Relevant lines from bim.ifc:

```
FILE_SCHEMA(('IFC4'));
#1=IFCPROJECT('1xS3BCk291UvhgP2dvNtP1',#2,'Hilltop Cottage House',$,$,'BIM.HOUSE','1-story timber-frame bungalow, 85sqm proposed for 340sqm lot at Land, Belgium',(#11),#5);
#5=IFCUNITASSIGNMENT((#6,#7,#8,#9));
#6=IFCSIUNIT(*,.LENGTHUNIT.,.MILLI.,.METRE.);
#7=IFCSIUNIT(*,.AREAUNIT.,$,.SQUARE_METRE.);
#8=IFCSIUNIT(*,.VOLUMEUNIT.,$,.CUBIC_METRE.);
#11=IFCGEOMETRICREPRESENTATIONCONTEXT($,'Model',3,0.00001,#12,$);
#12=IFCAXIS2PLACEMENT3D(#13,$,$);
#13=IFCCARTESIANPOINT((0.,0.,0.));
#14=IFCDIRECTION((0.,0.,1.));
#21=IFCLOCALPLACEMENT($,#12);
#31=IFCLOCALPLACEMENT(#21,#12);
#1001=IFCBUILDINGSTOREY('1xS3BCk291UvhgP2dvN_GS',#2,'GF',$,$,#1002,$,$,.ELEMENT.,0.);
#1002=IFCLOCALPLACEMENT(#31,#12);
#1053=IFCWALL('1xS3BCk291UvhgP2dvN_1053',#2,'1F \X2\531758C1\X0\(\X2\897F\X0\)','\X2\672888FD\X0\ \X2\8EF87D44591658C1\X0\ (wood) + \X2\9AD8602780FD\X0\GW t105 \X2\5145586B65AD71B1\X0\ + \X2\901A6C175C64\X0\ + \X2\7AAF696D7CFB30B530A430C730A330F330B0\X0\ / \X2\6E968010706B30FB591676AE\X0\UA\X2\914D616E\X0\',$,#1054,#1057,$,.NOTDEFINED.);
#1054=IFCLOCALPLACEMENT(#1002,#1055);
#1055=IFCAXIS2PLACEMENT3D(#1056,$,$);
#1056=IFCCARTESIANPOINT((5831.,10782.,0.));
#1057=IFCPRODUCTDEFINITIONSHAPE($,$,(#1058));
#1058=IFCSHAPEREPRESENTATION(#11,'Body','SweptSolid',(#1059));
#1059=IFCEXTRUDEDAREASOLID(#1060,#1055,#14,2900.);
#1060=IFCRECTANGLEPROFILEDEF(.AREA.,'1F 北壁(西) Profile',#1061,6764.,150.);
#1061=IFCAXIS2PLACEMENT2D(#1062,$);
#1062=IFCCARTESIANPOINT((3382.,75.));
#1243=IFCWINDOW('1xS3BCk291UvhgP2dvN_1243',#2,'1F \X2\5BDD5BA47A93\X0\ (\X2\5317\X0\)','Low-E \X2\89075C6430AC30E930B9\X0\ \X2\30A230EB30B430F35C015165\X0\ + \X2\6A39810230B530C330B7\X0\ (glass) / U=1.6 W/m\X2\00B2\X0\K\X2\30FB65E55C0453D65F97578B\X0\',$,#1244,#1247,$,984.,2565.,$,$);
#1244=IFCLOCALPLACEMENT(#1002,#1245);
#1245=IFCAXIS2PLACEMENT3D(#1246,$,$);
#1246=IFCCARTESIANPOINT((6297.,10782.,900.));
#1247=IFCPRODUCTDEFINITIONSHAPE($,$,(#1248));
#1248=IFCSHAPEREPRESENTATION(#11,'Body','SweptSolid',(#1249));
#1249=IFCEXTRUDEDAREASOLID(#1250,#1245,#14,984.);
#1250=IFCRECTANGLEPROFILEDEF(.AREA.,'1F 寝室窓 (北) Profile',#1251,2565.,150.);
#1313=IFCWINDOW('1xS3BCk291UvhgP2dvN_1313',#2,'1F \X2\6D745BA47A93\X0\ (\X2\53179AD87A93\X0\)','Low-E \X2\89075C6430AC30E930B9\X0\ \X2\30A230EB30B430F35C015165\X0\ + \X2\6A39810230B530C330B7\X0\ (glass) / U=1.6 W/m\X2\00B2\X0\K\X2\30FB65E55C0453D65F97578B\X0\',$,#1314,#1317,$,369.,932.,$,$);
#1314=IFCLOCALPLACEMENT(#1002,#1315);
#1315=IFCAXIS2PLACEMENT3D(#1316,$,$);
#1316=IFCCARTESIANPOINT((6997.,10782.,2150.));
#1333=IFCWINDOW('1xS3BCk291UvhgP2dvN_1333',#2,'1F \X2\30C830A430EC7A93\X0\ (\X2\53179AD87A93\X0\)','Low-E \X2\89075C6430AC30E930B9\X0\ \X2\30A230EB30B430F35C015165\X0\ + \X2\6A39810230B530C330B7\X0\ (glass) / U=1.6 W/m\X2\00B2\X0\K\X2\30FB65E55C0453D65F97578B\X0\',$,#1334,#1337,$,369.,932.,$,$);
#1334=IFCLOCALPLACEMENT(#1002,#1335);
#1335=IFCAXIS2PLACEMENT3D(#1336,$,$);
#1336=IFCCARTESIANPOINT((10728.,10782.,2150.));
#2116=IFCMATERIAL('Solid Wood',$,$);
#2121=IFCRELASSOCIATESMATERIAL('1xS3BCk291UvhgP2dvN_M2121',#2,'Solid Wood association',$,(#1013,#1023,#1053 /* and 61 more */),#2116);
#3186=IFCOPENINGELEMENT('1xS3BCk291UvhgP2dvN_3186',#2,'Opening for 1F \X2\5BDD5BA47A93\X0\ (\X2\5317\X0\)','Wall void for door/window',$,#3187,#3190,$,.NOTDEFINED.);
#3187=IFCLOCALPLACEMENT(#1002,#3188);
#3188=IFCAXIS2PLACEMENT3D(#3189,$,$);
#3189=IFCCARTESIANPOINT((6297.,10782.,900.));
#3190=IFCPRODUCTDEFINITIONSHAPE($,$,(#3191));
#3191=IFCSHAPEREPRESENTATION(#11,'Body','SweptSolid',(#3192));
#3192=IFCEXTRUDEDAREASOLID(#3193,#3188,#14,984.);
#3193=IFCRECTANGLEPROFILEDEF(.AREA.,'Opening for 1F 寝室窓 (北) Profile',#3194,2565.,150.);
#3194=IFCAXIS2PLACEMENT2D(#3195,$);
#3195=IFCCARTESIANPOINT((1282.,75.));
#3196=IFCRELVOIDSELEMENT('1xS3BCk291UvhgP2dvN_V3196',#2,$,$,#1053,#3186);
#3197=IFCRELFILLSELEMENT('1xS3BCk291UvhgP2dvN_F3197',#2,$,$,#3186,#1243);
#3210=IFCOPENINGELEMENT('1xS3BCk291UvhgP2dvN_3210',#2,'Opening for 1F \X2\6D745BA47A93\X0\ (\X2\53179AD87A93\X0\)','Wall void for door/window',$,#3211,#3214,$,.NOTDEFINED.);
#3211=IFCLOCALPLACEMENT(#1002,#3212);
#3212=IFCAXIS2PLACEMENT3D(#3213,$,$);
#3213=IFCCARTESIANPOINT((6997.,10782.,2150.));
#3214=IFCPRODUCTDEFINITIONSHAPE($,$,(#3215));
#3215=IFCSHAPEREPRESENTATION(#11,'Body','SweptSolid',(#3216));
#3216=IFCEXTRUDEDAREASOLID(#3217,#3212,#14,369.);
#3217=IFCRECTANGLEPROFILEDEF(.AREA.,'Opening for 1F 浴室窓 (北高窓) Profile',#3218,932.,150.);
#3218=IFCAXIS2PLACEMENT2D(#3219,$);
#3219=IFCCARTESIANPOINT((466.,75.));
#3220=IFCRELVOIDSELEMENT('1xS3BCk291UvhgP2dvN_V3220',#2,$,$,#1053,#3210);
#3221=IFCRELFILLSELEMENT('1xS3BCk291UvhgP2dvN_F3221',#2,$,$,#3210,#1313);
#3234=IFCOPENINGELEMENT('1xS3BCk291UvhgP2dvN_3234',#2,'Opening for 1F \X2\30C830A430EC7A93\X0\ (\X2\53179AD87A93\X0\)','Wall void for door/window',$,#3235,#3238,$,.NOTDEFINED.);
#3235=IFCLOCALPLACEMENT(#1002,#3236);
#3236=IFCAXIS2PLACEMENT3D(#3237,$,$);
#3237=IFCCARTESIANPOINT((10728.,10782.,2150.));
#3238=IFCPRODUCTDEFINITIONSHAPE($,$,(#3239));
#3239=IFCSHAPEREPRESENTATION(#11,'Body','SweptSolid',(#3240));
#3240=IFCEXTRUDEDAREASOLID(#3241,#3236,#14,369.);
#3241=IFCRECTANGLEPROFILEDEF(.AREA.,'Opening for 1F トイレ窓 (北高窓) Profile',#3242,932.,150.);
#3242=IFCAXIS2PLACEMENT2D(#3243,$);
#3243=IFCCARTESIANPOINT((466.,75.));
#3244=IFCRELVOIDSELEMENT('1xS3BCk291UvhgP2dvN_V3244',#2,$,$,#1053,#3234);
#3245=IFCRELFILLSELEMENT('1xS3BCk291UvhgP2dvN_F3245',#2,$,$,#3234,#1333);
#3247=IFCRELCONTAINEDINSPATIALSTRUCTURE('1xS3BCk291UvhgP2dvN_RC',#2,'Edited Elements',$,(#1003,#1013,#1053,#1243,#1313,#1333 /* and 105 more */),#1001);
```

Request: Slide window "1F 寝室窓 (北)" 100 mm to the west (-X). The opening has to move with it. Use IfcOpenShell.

```python
import ifcopenshell
import ifcopenshell.api.geometry
import ifcopenshell.util.placement

model = ifcopenshell.open("bim.ifc")

window = model.by_guid("1xS3BCk291UvhgP2dvN_1243")
opening = window.FillsVoids[0].RelatingOpeningElement
wall = opening.VoidsElements[0].RelatingBuildingElement

wall_matrix = ifcopenshell.util.placement.get_local_placement(wall.ObjectPlacement)
shift = wall_matrix[:3, 0] * -100.0
before = ifcopenshell.util.placement.get_local_placement(window.ObjectPlacement)[:3, 3].copy()

# The window is not placed relative to its opening, so move both.
for product in (opening, window):
    matrix = ifcopenshell.util.placement.get_local_placement(product.ObjectPlacement)
    matrix[:3, 3] += shift
    ifcopenshell.api.geometry.edit_object_placement(model, product=product, matrix=matrix, is_si=False)

after = ifcopenshell.util.placement.get_local_placement(window.ObjectPlacement)[:3, 3]
print("window moved by", (after - before).round(3) + 0.0)

model.write("bim_rev.ifc")
```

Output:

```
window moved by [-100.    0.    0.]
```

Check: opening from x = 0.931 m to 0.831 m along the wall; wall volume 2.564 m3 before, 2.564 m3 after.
